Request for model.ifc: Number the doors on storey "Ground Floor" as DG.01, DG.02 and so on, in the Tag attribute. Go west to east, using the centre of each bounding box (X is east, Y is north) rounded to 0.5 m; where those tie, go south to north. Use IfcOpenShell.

First a look at what the model holds.

```python
import ifcopenshell
import ifcopenshell.util.element
import ifcopenshell.util.placement

model = ifcopenshell.open("model.ifc")
print(model.schema)
storey = next(s for s in model.by_type("IfcBuildingStorey") if s.Name == "Ground Floor")
doors = [e for e in ifcopenshell.util.element.get_decomposition(storey) if e.is_a("IfcDoor")]
for e in sorted(doors, key=lambda e: e.id()):
    origin = ifcopenshell.util.placement.get_local_placement(e.ObjectPlacement)[:3, 3]
    print(e.id(), e.Tag, e.Name, origin.round(2) + 0.0, sep=" | ")
```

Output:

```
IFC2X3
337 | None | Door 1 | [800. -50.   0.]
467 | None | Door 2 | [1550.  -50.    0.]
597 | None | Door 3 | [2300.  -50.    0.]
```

```python
import ifcopenshell
import ifcopenshell.geom
import ifcopenshell.util.element
import ifcopenshell.util.shape

model = ifcopenshell.open("model.ifc")
settings = ifcopenshell.geom.settings()
settings.set("use-world-coords", True)


def centre(element):
    shape = ifcopenshell.geom.create_shape(settings, element)
    return ifcopenshell.util.shape.get_bbox_centroid(shape.geometry)


storey = next(s for s in model.by_type("IfcBuildingStorey") if s.Name == "Ground Floor")
doors = [e for e in ifcopenshell.util.element.get_decomposition(storey) if e.is_a("IfcDoor")]

# Insertion points can sit at a corner or the storey origin, so sort by the geometry (in metres).
centres = {e: centre(e) for e in doors}
doors.sort(key=lambda e: (round(centres[e][0] / 0.5), centres[e][1]))

for i, e in enumerate(doors, start=1):
    number = f"DG.{i:02d}"
    e.Tag = number
    print(e.id(), number)

model.write("model_v2.ifc")
```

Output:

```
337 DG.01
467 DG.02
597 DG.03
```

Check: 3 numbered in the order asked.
